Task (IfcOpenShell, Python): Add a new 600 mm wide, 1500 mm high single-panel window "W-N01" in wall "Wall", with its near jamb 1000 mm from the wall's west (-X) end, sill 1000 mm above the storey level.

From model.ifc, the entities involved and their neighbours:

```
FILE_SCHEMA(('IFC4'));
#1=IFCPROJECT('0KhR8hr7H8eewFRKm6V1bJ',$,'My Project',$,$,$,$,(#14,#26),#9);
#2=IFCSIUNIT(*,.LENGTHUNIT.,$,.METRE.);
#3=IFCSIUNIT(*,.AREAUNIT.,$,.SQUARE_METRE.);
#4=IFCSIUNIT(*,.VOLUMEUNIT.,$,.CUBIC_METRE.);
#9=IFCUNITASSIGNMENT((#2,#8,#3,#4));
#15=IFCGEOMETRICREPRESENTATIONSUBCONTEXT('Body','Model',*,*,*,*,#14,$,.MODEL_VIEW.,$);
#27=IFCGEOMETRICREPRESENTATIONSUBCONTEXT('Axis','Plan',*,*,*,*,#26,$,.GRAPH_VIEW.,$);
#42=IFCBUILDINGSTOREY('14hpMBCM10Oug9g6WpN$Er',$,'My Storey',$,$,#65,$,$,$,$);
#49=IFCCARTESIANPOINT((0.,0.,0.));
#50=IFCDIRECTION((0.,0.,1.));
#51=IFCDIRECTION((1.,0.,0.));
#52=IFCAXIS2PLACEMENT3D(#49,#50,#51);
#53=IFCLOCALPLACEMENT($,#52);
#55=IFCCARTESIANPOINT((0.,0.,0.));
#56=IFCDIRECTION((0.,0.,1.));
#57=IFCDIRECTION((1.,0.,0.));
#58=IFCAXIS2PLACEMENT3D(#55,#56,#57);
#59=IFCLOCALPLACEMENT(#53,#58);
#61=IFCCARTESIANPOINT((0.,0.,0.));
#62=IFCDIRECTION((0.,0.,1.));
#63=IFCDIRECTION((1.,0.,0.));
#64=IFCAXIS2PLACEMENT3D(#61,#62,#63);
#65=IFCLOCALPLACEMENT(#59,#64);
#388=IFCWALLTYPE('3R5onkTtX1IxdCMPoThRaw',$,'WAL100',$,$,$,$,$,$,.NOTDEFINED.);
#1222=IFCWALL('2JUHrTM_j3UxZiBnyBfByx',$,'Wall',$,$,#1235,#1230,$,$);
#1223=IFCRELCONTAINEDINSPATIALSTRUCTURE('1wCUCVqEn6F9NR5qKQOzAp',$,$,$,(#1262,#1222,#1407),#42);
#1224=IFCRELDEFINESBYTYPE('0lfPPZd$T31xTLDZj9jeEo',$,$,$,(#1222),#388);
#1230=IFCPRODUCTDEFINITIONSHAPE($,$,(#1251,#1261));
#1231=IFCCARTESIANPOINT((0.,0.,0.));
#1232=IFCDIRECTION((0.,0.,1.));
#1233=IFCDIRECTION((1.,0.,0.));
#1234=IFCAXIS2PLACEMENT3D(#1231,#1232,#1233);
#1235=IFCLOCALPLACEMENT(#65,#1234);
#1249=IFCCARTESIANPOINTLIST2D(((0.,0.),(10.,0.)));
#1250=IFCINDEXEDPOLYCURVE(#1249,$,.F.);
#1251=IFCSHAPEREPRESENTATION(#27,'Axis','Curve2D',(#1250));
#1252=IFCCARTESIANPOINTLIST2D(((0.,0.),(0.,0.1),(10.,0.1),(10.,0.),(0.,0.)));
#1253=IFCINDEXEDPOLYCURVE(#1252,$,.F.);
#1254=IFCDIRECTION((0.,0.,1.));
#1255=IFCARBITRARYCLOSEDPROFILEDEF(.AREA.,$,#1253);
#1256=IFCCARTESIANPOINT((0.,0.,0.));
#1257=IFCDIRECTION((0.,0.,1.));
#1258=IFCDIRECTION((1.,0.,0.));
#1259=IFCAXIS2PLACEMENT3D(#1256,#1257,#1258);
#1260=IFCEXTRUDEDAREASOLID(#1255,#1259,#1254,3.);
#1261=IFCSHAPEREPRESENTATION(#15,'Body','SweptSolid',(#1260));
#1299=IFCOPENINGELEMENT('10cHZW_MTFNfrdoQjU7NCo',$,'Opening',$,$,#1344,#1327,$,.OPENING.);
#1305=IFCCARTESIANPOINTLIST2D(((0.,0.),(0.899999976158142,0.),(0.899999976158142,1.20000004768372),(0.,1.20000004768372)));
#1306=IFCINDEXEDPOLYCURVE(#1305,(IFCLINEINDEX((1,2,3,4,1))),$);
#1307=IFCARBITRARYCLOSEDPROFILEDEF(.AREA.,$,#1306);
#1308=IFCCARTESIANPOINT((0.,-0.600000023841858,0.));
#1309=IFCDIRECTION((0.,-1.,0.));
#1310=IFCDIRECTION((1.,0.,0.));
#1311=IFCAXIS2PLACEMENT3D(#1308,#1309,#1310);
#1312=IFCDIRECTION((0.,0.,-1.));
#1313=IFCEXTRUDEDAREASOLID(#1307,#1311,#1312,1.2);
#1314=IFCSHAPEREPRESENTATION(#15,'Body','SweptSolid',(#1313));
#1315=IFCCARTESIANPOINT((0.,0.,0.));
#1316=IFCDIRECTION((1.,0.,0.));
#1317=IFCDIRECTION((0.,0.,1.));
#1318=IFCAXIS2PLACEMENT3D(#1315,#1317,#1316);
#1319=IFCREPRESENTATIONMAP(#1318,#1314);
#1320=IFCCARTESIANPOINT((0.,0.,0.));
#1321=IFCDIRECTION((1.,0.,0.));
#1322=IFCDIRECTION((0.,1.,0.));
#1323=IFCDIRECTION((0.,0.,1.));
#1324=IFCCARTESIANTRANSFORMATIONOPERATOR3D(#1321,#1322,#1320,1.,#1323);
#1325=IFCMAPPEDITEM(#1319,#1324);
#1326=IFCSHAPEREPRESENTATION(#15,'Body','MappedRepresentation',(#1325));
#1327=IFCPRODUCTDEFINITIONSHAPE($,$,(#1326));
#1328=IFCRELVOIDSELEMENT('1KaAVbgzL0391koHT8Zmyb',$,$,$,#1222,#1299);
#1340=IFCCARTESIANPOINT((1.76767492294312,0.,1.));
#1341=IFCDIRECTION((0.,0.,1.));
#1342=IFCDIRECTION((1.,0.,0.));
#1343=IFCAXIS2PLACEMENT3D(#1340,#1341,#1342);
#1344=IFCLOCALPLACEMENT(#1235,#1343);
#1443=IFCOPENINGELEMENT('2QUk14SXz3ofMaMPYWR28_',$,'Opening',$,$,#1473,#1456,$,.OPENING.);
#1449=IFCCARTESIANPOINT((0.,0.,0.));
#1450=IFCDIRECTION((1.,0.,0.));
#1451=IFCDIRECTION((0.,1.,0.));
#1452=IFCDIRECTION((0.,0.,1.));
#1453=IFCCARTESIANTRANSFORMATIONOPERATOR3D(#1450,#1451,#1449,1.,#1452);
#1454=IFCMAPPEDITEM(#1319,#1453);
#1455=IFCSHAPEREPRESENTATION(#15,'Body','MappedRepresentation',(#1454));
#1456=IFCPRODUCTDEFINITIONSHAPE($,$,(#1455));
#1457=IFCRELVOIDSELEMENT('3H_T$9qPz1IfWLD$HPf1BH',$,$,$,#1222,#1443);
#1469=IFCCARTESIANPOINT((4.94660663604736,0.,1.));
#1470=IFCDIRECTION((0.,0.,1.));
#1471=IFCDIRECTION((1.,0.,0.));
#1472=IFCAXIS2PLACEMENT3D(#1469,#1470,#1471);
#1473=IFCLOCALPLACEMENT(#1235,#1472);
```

```python
import numpy as np
import ifcopenshell
import ifcopenshell.api.feature
import ifcopenshell.api.geometry
import ifcopenshell.api.root
import ifcopenshell.api.spatial
import ifcopenshell.geom
import ifcopenshell.util.element
import ifcopenshell.util.placement
import ifcopenshell.util.representation
import ifcopenshell.util.shape
import ifcopenshell.util.unit

model = ifcopenshell.open("model.ifc")
unit_scale = ifcopenshell.util.unit.calculate_unit_scale(model)
settings = ifcopenshell.geom.settings()


def volume(element):
    """Net volume in cubic metres, openings subtracted."""
    shape = ifcopenshell.geom.create_shape(settings, element)
    return ifcopenshell.util.shape.get_volume(shape.geometry)


wall = model.by_guid("2JUHrTM_j3UxZiBnyBfByx")
storey = ifcopenshell.util.element.get_container(wall, ifc_class="IfcBuildingStorey")
context = ifcopenshell.util.representation.get_context(model, "Model", "Body", "MODEL_VIEW")
before = volume(wall)

width, height, from_end, sill = 0.6, 1.5, 1, 1  # metres

# The wall runs along its own X axis, and the end named is its -X end.
wall_shape = ifcopenshell.geom.create_shape(settings, wall)
x, y, z = ifcopenshell.util.shape.get_vertices(wall_shape.geometry).T
start = x.min() + from_end
face, thickness = float(y.min()), float(y.max() - y.min())
wall_matrix = ifcopenshell.util.placement.get_local_placement(wall.ObjectPlacement)
level = ifcopenshell.util.placement.get_local_placement(storey.ObjectPlacement)[2, 3]


def in_wall(x, y):
    """Placement at x, y metres in the wall's axes, at sill height."""
    matrix = wall_matrix.copy()
    matrix[:, 3] = wall_matrix @ np.array([x / unit_scale, y / unit_scale, 0.0, 1.0])
    matrix[2, 3] = level + sill / unit_scale
    return matrix


# Opening: a box that overshoots both wall faces by 50 mm.
opening = ifcopenshell.api.root.create_entity(model, ifc_class="IfcOpeningElement", predefined_type="OPENING")
box = ifcopenshell.api.geometry.add_wall_representation(
    model, context=context, length=width, height=height, thickness=thickness + 0.1
)
ifcopenshell.api.geometry.assign_representation(model, product=opening, representation=box)
ifcopenshell.api.geometry.edit_object_placement(model, product=opening, matrix=in_wall(start, face - 0.05), is_si=False)
ifcopenshell.api.feature.add_feature(model, feature=opening, element=wall)

window = ifcopenshell.api.root.create_entity(model, ifc_class="IfcWindow", name="W-N01", predefined_type="WINDOW")
window.OverallWidth, window.OverallHeight = width / unit_scale, height / unit_scale
window.PartitioningType = "SINGLE_PANEL"
body = ifcopenshell.api.geometry.add_window_representation(
    model,
    context=context,
    overall_width=window.OverallWidth,
    overall_height=window.OverallHeight,
    partition_type="SINGLE_PANEL",
)
ifcopenshell.api.geometry.assign_representation(model, product=window, representation=body)
ifcopenshell.api.spatial.assign_container(model, products=[window], relating_structure=storey)
ifcopenshell.api.feature.add_filling(model, opening=opening, element=window)

# Centre the window in the wall's thickness.
ifcopenshell.api.geometry.edit_object_placement(model, product=window, matrix=in_wall(start, face), is_si=False)
window_shape = ifcopenshell.geom.create_shape(settings, window)
depth = ifcopenshell.util.shape.get_vertices(window_shape.geometry)[:, 1]
offset = face + thickness / 2 - (depth.min() + depth.max()) / 2
ifcopenshell.api.geometry.edit_object_placement(model, product=window, matrix=in_wall(start, offset), is_si=False)

after = volume(wall)

print(f"wall volume {before:.3f} -> {after:.3f} m3")

model.write("model_v2.ifc")
```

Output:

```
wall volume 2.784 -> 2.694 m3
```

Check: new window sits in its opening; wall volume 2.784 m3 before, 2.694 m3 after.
